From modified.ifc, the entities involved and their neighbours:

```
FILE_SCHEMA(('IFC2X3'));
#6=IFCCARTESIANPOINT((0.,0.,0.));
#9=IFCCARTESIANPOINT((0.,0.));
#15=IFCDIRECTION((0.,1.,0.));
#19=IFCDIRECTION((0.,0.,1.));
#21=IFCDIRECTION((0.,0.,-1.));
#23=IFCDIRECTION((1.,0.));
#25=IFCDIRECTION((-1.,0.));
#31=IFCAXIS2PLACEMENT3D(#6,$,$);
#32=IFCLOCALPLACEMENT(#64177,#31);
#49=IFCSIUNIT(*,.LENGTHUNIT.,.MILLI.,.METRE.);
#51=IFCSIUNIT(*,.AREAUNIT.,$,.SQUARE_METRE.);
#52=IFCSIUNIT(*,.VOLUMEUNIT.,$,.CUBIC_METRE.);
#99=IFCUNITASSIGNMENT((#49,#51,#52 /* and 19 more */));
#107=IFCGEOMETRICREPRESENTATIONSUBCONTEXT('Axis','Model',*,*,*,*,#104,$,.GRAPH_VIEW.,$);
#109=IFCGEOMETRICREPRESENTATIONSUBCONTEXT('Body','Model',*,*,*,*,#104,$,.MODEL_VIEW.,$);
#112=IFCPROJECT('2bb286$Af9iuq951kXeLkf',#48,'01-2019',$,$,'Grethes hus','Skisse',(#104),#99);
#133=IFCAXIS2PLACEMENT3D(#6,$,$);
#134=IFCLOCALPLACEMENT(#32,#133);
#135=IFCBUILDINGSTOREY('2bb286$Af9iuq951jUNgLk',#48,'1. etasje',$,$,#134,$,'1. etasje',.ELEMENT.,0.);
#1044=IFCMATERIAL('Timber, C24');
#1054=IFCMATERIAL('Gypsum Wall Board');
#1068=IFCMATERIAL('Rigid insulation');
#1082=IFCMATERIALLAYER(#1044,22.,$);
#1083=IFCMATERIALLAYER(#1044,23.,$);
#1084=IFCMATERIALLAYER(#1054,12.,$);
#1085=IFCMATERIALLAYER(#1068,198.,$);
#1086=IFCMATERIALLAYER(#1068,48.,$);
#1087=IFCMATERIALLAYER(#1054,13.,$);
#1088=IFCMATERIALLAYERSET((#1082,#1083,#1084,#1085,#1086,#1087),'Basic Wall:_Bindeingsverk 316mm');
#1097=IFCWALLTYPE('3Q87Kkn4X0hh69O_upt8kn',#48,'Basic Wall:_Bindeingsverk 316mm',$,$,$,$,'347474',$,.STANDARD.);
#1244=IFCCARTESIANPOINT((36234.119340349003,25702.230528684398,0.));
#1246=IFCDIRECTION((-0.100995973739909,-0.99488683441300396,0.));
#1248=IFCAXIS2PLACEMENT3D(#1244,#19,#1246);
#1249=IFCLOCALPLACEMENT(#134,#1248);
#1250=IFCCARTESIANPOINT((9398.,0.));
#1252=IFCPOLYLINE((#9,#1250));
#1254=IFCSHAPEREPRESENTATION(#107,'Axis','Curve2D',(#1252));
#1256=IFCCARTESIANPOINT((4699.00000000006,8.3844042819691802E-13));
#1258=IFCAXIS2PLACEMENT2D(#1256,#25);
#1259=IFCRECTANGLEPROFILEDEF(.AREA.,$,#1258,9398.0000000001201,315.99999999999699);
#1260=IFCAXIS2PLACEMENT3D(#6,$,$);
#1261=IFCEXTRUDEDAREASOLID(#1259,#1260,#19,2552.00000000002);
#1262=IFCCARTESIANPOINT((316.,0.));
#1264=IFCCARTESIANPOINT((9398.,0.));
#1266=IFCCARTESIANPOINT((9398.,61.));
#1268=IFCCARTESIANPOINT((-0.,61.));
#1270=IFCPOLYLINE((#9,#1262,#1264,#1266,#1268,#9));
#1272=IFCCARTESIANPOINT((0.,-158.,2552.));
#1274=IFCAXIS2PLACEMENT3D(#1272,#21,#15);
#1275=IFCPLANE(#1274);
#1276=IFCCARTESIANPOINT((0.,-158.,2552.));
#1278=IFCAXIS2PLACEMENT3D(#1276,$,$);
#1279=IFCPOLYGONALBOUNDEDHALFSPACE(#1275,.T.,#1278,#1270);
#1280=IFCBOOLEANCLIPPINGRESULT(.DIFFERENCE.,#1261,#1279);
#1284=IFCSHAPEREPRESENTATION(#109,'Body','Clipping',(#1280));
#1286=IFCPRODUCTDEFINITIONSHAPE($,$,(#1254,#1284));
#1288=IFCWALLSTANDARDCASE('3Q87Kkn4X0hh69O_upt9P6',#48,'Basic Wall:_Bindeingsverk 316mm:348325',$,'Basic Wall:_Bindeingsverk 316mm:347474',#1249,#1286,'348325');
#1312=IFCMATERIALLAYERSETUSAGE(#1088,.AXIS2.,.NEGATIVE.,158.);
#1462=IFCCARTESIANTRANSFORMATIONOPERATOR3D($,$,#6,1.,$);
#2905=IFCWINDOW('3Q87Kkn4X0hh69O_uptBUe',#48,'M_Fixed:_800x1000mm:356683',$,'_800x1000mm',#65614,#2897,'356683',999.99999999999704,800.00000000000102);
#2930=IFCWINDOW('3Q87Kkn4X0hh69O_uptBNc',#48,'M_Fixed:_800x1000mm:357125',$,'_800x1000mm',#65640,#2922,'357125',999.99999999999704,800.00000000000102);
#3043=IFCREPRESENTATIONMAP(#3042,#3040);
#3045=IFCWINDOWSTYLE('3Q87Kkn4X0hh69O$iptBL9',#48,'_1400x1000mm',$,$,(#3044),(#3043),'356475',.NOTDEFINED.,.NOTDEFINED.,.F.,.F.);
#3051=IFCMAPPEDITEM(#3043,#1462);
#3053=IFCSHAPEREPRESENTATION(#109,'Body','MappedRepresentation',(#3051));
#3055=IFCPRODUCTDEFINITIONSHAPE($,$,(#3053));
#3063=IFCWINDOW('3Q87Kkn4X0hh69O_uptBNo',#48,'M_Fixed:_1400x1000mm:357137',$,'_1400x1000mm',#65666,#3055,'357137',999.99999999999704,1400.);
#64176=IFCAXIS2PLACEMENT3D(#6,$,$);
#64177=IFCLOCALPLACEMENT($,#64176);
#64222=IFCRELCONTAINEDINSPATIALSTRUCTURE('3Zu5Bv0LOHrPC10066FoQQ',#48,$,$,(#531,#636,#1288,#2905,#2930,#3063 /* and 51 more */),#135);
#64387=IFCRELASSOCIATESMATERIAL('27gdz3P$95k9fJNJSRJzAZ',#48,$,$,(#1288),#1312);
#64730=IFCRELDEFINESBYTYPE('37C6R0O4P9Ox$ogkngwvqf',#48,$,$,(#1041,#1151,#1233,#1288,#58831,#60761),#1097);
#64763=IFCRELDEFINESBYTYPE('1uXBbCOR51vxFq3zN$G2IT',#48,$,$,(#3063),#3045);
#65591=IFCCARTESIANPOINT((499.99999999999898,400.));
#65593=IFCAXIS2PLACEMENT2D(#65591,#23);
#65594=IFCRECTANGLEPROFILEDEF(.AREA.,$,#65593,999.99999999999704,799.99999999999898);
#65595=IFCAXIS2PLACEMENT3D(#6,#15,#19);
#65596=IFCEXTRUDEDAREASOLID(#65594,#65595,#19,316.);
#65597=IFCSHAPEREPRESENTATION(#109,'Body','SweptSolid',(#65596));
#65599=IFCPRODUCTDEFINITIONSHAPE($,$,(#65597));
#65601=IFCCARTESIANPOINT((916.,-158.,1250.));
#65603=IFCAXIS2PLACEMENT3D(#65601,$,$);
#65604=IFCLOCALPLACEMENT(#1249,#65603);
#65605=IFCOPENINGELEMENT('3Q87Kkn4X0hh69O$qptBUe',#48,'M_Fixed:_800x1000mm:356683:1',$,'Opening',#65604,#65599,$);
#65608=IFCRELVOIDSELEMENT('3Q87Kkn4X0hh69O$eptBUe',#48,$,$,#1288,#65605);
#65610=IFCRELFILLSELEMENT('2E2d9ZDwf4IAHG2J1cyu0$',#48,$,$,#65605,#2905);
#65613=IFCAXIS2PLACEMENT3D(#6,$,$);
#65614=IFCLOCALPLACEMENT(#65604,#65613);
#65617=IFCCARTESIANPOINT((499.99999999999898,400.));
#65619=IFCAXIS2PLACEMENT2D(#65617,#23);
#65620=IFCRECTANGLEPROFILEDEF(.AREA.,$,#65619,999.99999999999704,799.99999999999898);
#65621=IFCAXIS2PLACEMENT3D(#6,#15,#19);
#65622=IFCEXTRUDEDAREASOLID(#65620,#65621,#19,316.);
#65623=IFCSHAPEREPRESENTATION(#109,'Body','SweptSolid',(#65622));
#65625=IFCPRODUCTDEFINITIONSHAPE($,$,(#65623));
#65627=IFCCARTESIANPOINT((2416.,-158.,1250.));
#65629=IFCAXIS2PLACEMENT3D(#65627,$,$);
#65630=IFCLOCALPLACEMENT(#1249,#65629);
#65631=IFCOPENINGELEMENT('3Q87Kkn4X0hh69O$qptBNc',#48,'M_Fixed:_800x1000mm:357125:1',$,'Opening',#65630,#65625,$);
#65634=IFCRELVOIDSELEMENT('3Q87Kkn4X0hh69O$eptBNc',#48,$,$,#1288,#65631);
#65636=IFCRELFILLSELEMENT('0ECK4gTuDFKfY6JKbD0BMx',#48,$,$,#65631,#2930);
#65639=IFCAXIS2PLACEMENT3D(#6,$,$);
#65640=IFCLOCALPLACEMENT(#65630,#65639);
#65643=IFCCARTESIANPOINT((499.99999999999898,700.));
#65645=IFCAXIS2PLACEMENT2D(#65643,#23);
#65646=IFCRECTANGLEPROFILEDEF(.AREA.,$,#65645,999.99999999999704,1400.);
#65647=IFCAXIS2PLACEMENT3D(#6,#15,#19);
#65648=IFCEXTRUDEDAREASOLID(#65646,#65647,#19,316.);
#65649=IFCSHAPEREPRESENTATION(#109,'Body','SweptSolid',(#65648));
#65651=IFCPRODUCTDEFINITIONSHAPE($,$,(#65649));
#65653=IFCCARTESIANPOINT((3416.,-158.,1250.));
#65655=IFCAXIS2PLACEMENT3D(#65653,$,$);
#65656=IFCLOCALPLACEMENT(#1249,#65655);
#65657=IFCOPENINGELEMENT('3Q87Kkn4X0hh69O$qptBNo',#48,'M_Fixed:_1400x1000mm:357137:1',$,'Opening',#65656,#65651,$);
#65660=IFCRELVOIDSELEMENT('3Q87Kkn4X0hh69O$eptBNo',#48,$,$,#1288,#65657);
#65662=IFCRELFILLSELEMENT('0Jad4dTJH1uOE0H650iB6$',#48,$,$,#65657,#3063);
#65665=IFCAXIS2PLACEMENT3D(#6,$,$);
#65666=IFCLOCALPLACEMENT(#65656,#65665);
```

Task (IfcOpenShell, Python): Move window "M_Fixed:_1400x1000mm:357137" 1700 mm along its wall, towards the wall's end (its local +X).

```python
import ifcopenshell
import ifcopenshell.api.geometry
import ifcopenshell.util.placement

model = ifcopenshell.open("modified.ifc")

window = model.by_id(3063)
opening = window.FillsVoids[0].RelatingOpeningElement
wall = opening.VoidsElements[0].RelatingBuildingElement

wall_matrix = ifcopenshell.util.placement.get_local_placement(wall.ObjectPlacement)
shift = wall_matrix[:3, 0] * 1700.0
before = ifcopenshell.util.placement.get_local_placement(window.ObjectPlacement)[:3, 3].copy()

# The window is placed relative to its opening, so it follows when the opening moves.
matrix = ifcopenshell.util.placement.get_local_placement(opening.ObjectPlacement)
matrix[:3, 3] += shift
ifcopenshell.api.geometry.edit_object_placement(
    model, product=opening, matrix=matrix, is_si=False, should_transform_children=True
)

after = ifcopenshell.util.placement.get_local_placement(window.ObjectPlacement)[:3, 3]
print("window moved by", (after - before).round(3) + 0.0)

model.write("modified_updated.ifc")
```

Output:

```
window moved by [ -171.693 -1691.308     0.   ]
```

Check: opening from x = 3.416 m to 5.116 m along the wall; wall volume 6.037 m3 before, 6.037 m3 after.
